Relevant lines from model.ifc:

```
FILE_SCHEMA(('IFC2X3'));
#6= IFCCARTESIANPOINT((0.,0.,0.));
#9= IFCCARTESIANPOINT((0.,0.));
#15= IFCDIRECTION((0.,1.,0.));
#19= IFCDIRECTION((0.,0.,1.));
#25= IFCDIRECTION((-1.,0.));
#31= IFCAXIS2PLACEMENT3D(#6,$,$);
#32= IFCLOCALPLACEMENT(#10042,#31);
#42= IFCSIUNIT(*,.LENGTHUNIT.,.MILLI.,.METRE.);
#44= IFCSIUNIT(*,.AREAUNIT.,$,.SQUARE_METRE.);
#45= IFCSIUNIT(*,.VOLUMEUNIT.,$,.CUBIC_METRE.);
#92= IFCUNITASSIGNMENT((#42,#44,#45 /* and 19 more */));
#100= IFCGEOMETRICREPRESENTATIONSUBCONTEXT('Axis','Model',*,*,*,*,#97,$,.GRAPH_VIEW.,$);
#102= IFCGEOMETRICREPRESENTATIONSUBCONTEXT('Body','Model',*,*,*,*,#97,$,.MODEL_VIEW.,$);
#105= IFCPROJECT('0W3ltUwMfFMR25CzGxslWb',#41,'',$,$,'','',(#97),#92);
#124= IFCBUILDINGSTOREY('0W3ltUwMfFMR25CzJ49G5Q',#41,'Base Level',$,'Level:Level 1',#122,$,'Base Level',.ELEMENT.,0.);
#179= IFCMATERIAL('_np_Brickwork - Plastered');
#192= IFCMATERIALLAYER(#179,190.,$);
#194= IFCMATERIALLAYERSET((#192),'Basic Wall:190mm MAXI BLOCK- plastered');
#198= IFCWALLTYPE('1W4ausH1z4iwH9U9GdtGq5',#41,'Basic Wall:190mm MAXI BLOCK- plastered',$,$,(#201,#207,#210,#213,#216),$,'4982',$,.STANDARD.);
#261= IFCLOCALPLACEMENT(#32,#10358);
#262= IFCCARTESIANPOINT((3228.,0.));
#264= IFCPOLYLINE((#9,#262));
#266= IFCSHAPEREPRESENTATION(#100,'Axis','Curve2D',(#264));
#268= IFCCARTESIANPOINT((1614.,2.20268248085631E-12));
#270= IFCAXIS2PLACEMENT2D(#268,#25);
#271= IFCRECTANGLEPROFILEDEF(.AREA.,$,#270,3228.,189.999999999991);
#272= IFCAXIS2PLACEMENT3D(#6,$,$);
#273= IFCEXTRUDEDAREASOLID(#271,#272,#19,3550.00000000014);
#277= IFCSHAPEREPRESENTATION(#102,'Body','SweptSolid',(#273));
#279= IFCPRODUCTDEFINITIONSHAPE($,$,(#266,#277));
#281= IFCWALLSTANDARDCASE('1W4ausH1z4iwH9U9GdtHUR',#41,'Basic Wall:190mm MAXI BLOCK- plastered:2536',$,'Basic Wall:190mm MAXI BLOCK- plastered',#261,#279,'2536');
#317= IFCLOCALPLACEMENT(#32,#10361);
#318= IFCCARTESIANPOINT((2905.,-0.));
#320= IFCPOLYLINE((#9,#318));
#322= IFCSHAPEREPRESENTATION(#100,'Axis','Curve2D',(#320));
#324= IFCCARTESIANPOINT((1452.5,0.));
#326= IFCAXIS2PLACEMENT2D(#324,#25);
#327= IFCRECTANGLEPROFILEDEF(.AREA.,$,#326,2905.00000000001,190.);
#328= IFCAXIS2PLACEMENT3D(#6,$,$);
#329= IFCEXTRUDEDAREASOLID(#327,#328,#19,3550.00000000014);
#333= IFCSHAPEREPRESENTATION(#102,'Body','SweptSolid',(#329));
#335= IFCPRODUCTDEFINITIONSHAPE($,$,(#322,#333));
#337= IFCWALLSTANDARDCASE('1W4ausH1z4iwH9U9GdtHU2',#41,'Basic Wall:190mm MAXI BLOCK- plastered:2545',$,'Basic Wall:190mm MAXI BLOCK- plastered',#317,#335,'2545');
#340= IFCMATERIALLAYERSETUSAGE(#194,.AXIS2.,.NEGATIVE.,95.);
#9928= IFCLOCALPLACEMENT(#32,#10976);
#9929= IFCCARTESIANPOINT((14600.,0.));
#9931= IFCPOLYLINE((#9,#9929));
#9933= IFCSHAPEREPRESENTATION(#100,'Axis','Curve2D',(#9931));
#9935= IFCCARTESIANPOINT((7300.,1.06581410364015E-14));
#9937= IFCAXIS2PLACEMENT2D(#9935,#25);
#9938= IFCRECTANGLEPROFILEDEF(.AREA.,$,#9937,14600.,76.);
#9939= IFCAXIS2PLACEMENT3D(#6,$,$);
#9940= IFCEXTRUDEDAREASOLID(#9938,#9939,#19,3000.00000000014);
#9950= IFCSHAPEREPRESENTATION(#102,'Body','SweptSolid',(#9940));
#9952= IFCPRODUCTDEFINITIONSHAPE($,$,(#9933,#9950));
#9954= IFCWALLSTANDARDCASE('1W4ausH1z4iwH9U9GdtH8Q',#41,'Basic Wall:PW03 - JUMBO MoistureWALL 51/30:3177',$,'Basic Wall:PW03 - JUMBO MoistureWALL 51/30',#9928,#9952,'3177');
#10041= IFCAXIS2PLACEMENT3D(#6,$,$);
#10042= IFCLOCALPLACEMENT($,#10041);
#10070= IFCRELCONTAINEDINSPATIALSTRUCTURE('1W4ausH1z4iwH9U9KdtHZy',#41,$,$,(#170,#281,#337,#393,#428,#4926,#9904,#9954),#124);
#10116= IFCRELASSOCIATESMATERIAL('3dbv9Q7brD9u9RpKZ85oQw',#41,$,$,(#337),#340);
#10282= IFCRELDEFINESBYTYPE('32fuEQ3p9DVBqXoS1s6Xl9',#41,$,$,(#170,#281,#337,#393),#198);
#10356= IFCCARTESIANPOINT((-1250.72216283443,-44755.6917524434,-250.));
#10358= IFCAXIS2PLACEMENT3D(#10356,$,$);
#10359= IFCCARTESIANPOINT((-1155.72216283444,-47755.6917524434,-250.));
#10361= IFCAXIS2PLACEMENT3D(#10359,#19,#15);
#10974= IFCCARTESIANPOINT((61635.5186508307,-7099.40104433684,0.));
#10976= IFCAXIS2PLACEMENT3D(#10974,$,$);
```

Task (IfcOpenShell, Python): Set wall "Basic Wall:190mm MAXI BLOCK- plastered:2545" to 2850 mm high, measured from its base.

```python
import ifcopenshell
import ifcopenshell.geom
import ifcopenshell.util.representation
import ifcopenshell.util.shape

model = ifcopenshell.open("model.ifc")
settings = ifcopenshell.geom.settings()


def volume(element):
    """Net volume in cubic metres, openings subtracted."""
    shape = ifcopenshell.geom.create_shape(settings, element)
    return ifcopenshell.util.shape.get_volume(shape.geometry)


wall = model.by_id(337)
before = volume(wall)

body = ifcopenshell.util.representation.get_representation(wall, "Model", "Body")
solid = body.Items[0]
old_height = solid.Depth
solid.Depth = 2850.0
after = volume(wall)

print(f"height {old_height:g} -> {solid.Depth:g}, volume {before:.3f} -> {after:.3f} m3")

model.write("model_updated.ifc")
```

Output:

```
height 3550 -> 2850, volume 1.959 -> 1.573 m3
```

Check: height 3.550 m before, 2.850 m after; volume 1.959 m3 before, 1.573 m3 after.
